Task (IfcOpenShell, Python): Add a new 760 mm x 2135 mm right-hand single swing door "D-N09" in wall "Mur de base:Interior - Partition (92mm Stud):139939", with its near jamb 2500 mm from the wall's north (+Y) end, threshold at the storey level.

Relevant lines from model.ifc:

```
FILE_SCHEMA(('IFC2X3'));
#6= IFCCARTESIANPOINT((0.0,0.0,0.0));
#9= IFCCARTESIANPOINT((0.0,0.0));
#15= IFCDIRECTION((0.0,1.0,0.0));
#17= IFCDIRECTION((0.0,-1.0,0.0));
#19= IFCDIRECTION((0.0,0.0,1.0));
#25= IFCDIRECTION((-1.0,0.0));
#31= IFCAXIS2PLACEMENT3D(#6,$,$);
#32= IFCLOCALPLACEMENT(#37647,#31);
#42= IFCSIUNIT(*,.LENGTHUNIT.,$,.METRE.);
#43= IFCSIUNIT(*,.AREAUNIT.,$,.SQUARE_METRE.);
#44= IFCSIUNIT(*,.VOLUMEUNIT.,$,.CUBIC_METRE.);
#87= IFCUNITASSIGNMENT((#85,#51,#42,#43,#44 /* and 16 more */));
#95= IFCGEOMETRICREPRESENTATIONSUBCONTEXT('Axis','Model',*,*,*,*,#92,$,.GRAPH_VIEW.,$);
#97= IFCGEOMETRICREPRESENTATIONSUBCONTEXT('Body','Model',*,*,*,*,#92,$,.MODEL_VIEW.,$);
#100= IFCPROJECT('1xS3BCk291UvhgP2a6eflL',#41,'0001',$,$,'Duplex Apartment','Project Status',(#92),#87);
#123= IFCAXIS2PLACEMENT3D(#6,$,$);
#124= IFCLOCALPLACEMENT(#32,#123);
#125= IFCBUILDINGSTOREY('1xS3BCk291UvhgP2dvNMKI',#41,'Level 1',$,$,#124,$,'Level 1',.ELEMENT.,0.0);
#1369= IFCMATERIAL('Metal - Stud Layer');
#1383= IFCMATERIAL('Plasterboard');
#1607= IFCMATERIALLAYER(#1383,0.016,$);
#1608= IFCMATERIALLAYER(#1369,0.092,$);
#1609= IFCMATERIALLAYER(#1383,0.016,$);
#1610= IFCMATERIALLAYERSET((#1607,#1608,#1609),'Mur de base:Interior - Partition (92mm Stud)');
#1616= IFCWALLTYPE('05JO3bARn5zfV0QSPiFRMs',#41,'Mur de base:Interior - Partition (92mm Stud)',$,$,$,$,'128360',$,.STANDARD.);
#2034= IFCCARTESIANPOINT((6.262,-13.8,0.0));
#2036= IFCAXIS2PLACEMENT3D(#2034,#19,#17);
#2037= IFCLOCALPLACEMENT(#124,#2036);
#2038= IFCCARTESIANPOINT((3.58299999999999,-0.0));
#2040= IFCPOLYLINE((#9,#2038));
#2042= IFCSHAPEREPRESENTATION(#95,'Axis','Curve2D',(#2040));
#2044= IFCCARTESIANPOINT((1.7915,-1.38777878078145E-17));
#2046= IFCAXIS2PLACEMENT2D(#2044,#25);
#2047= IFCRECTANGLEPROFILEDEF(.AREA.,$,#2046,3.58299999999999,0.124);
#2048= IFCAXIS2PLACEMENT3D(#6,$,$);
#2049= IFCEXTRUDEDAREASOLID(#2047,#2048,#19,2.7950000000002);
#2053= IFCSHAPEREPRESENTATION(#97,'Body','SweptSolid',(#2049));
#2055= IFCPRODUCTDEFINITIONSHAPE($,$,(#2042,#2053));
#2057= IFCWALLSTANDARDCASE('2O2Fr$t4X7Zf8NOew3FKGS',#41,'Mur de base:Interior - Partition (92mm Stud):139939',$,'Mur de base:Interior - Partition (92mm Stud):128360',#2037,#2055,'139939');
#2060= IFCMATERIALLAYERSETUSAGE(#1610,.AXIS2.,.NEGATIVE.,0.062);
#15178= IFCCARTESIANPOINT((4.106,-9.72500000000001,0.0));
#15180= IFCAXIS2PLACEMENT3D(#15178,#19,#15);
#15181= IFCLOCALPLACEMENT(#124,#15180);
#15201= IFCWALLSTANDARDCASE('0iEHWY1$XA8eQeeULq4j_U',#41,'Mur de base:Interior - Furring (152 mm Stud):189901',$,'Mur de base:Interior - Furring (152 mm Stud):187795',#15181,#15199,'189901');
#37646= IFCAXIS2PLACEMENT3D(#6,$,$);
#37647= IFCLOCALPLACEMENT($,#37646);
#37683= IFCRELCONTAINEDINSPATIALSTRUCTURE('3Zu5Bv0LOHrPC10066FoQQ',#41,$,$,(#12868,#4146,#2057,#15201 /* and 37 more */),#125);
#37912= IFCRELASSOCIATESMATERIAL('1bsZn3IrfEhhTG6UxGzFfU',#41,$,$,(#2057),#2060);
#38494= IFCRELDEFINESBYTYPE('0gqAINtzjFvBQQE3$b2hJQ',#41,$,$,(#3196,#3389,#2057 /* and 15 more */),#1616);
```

```python
import numpy as np
import ifcopenshell
import ifcopenshell.api.feature
import ifcopenshell.api.geometry
import ifcopenshell.api.root
import ifcopenshell.api.spatial
import ifcopenshell.api.type
import ifcopenshell.geom
import ifcopenshell.util.element
import ifcopenshell.util.placement
import ifcopenshell.util.representation
import ifcopenshell.util.shape
import ifcopenshell.util.unit

model = ifcopenshell.open("model.ifc")
unit_scale = ifcopenshell.util.unit.calculate_unit_scale(model)
settings = ifcopenshell.geom.settings()


def volume(element):
    """Net volume in cubic metres, openings subtracted."""
    shape = ifcopenshell.geom.create_shape(settings, element)
    return ifcopenshell.util.shape.get_volume(shape.geometry)


wall = model.by_id(2057)
storey = ifcopenshell.util.element.get_container(wall, ifc_class="IfcBuildingStorey")
context = ifcopenshell.util.representation.get_context(model, "Model", "Body", "MODEL_VIEW")
before = volume(wall)

width, height, from_end, sill = 0.76, 2.135, 2.5, 0.0  # metres

# The wall runs along its own X axis, and the end named is its -X end.
wall_shape = ifcopenshell.geom.create_shape(settings, wall)
x, y, z = ifcopenshell.util.shape.get_vertices(wall_shape.geometry).T
start = x.min() + from_end
face, thickness = float(y.min()), float(y.max() - y.min())
wall_matrix = ifcopenshell.util.placement.get_local_placement(wall.ObjectPlacement)
level = ifcopenshell.util.placement.get_local_placement(storey.ObjectPlacement)[2, 3]


def in_wall(x, y):
    """Placement at x, y metres in the wall's axes, at sill height."""
    matrix = wall_matrix.copy()
    matrix[:, 3] = wall_matrix @ np.array([x / unit_scale, y / unit_scale, 0.0, 1.0])
    matrix[2, 3] = level + sill / unit_scale
    return matrix


# Opening: a box that overshoots both wall faces by 50 mm.
opening = ifcopenshell.api.root.create_entity(model, ifc_class="IfcOpeningElement")
box = ifcopenshell.api.geometry.add_wall_representation(
    model, context=context, length=width, height=height, thickness=thickness + 0.1
)
ifcopenshell.api.geometry.assign_representation(model, product=opening, representation=box)
ifcopenshell.api.geometry.edit_object_placement(model, product=opening, matrix=in_wall(start, face - 0.05), is_si=False)
ifcopenshell.api.feature.add_feature(model, feature=opening, element=wall)

door = ifcopenshell.api.root.create_entity(model, ifc_class="IfcDoor", name="D-N09")
door.OverallWidth, door.OverallHeight = width / unit_scale, height / unit_scale
body = ifcopenshell.api.geometry.add_door_representation(
    model,
    context=context,
    overall_width=door.OverallWidth,
    overall_height=door.OverallHeight,
    operation_type="SINGLE_SWING_RIGHT",
    lining_properties={"LiningDepth": thickness / unit_scale, "ThresholdDepth": thickness / unit_scale},
)
ifcopenshell.api.geometry.assign_representation(model, product=door, representation=body)
ifcopenshell.api.spatial.assign_container(model, products=[door], relating_structure=storey)
fills = ifcopenshell.api.feature.add_filling(model, opening=opening, element=door)
fills.OwnerHistory = door.OwnerHistory  # required in IFC2X3

# IFC2X3 keeps the operation on the door style.
style = ifcopenshell.api.root.create_entity(model, ifc_class="IfcDoorStyle", name="D-N09")
style.OperationType, style.ConstructionType = "SINGLE_SWING_RIGHT", "NOTDEFINED"
style.ParameterTakesPrecedence = style.Sizeable = False
ifcopenshell.api.type.assign_type(model, related_objects=[door], relating_type=style)

# The lining spans the wall, so the door starts at the wall face.
ifcopenshell.api.geometry.edit_object_placement(model, product=door, matrix=in_wall(start, face), is_si=False)

after = volume(wall)

print(f"wall volume {before:.3f} -> {after:.3f} m3")

model.write("model-out.ifc")
```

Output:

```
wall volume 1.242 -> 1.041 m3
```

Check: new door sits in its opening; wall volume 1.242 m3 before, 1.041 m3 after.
